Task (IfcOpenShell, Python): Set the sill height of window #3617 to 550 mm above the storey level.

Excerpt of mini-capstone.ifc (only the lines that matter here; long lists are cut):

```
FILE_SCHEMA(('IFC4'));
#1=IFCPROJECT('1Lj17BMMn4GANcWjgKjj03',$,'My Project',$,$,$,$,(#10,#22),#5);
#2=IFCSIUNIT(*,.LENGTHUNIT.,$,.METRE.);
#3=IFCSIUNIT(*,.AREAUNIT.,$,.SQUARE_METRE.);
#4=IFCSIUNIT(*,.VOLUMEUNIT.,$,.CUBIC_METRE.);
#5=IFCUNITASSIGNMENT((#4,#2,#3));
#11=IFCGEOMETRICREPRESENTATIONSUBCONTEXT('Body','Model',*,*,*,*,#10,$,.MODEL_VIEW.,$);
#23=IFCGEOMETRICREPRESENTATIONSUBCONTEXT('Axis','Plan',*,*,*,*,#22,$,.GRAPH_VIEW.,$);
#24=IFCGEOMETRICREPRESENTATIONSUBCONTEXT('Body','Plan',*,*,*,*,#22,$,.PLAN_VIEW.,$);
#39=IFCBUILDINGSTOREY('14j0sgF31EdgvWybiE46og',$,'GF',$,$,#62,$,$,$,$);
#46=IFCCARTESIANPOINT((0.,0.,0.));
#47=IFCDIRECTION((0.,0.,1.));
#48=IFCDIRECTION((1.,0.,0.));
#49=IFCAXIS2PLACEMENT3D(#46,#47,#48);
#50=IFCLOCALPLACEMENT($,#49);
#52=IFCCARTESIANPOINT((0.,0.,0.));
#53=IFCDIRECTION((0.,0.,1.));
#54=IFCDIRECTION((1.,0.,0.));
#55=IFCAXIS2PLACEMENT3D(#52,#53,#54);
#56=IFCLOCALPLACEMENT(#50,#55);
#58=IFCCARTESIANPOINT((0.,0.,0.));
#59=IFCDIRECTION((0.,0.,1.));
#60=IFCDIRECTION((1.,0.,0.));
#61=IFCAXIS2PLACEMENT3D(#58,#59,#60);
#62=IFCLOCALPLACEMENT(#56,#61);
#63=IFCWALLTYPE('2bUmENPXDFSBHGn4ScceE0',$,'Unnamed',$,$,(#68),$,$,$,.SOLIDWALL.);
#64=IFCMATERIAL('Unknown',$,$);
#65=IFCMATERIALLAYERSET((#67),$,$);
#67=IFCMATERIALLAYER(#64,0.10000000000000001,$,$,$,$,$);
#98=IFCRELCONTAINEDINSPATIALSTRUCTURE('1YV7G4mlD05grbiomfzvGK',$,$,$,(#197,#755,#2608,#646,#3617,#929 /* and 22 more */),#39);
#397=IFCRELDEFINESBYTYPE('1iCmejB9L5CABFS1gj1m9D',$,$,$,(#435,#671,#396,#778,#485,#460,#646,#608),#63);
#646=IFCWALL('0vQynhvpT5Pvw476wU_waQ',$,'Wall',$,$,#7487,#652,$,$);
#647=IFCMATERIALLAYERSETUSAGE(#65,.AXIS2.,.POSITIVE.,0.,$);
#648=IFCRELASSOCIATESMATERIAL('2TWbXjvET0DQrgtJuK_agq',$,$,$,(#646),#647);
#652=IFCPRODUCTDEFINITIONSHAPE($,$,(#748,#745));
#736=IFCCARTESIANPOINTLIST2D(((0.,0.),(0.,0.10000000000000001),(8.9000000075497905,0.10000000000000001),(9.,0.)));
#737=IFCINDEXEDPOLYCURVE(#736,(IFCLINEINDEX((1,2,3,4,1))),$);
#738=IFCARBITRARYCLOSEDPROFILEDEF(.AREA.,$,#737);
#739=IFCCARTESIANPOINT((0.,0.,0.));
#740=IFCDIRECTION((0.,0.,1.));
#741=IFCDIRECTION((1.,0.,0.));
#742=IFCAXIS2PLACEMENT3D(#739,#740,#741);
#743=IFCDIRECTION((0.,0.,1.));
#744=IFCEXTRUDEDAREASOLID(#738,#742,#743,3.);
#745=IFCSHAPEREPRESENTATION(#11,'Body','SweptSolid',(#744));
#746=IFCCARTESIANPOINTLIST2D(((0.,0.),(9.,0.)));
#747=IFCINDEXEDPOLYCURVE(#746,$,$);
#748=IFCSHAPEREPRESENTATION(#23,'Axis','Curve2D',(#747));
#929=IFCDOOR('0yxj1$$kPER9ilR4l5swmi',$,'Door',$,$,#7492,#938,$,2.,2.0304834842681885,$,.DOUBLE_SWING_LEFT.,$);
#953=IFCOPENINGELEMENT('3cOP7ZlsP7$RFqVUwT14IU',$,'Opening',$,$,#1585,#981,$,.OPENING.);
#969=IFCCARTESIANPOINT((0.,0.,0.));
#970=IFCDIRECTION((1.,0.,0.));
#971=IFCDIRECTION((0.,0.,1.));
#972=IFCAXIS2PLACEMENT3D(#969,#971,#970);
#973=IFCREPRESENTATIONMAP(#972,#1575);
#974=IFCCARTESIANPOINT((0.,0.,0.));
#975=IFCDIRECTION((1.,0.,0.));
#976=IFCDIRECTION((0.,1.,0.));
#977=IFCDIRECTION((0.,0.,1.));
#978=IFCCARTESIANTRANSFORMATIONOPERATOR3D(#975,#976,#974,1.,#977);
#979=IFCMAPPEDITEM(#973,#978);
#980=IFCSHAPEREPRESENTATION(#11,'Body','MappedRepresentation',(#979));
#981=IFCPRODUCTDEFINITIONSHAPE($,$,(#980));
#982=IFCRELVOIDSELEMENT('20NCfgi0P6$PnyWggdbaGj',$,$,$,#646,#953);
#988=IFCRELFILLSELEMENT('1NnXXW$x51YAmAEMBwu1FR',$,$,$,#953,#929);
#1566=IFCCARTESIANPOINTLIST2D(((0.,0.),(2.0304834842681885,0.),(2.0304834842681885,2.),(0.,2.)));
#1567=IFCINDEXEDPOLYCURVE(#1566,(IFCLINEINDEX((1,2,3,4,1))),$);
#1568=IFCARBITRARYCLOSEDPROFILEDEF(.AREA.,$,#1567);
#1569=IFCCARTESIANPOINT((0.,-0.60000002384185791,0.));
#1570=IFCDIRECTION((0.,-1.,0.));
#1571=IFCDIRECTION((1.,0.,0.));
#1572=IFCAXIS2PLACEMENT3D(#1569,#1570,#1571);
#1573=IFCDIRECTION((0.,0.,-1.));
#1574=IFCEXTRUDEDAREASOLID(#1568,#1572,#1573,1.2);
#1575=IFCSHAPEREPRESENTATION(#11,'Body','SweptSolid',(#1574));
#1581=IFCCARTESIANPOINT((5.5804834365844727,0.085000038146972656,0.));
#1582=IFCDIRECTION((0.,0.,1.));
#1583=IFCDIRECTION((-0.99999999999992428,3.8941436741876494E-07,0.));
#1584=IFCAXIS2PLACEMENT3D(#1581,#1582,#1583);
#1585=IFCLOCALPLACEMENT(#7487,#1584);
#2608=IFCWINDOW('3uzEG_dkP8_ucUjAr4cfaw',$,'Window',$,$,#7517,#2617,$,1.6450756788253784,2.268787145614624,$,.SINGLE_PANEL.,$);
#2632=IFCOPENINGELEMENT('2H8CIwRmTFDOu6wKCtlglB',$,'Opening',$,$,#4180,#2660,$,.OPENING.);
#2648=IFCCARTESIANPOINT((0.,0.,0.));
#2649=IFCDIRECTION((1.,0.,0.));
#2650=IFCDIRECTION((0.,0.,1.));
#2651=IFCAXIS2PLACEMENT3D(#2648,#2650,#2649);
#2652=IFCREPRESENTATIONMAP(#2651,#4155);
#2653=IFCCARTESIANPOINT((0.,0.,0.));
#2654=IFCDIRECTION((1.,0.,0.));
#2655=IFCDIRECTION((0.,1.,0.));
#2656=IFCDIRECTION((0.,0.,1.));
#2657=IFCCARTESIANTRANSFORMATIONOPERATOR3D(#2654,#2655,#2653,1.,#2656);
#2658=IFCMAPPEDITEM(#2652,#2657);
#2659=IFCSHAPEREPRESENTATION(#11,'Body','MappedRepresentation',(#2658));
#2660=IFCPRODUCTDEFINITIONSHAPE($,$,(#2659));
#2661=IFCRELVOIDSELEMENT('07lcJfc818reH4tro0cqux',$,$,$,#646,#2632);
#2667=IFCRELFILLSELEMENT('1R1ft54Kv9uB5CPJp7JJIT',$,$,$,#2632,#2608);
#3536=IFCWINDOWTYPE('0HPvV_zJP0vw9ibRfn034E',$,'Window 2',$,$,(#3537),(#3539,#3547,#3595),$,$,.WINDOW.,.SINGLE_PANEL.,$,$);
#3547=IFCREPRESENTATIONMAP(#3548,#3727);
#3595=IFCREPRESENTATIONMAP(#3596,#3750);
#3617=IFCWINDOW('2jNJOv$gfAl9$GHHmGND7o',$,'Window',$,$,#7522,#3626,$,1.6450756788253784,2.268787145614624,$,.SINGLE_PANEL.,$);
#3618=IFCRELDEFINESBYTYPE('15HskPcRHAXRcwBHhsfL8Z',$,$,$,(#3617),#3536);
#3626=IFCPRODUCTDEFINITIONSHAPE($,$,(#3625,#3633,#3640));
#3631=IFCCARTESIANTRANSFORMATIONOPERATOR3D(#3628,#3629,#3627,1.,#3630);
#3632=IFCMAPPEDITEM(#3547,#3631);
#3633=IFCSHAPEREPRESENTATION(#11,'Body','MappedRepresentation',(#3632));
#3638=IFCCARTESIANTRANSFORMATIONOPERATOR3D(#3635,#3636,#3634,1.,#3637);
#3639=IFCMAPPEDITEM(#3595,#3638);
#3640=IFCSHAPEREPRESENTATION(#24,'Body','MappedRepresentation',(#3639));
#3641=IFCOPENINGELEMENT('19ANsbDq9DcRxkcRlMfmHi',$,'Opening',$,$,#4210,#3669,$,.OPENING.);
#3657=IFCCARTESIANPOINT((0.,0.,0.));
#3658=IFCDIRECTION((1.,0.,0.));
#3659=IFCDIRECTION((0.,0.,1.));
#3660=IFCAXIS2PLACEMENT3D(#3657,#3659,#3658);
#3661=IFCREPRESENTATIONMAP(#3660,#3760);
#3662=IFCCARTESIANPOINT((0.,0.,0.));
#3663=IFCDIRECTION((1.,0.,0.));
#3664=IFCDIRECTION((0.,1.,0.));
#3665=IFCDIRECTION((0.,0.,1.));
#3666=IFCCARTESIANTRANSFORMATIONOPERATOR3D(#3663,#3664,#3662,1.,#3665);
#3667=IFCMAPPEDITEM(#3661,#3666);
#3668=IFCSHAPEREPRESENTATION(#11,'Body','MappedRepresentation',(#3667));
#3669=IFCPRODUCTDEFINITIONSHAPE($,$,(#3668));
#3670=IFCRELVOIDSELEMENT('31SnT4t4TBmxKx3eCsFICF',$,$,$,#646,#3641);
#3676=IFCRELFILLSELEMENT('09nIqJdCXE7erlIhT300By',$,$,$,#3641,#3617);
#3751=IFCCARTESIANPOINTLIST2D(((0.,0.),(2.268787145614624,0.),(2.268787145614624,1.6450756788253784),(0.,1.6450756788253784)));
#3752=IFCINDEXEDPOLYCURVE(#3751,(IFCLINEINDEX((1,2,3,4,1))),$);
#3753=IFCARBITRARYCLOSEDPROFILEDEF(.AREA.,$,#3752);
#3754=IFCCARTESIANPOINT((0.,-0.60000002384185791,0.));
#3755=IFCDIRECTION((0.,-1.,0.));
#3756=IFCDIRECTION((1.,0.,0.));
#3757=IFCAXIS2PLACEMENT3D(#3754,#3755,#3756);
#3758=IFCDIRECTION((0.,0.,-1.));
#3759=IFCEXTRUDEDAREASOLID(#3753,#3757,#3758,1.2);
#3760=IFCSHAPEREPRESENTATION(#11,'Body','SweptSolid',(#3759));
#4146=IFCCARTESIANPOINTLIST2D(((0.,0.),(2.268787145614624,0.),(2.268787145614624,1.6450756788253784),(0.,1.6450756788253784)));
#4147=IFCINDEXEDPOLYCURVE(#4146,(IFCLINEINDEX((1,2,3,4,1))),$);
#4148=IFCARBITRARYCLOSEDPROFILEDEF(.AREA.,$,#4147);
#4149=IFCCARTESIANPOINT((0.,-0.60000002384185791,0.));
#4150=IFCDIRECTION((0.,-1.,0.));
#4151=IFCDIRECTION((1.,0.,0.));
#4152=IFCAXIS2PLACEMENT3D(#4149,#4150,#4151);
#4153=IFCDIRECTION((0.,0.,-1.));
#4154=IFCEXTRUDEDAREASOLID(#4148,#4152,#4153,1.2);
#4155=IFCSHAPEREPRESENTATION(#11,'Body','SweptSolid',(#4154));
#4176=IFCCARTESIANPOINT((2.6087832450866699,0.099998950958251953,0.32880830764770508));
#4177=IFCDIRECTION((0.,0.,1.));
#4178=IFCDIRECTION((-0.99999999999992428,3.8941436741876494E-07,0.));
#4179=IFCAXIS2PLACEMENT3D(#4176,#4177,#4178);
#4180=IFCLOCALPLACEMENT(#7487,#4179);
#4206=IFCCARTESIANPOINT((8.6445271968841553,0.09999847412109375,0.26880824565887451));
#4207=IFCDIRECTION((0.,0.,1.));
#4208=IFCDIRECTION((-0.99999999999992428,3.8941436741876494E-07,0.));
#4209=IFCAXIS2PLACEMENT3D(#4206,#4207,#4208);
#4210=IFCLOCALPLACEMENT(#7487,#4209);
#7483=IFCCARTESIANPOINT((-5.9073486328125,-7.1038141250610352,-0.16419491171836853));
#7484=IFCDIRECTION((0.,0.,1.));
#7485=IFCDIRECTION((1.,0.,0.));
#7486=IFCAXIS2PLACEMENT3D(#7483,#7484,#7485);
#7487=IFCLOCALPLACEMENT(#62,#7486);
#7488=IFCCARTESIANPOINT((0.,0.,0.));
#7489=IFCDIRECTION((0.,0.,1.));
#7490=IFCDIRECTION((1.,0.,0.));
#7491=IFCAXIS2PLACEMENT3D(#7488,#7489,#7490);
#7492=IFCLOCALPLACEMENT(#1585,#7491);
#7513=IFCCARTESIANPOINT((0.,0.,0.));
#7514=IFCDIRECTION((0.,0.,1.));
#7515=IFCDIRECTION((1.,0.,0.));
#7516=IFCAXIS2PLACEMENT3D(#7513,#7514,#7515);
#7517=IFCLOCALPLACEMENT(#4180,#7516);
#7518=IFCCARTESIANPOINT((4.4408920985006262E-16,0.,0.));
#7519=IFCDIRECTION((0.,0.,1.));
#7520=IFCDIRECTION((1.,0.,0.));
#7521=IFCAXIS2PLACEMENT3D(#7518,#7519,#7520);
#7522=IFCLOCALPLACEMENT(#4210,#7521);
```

```python
import numpy as np
import ifcopenshell
import ifcopenshell.api.geometry
import ifcopenshell.geom
import ifcopenshell.util.element
import ifcopenshell.util.placement
import ifcopenshell.util.shape
import ifcopenshell.util.unit

model = ifcopenshell.open("mini-capstone.ifc")
unit_scale = ifcopenshell.util.unit.calculate_unit_scale(model)

window = model.by_id(3617)
opening = window.FillsVoids[0].RelatingOpeningElement
storey = ifcopenshell.util.element.get_container(window, ifc_class="IfcBuildingStorey")
level = ifcopenshell.util.placement.get_local_placement(storey.ObjectPlacement)[2, 3]

# The opening's origin need not be at the sill, so measure its lowest point.
shape = ifcopenshell.geom.create_shape(ifcopenshell.geom.settings(), opening)
bottom = ifcopenshell.util.shape.get_shape_bottom_elevation(shape, shape.geometry) / unit_scale
dz = level + 0.55 / unit_scale - bottom

shift = np.array([0.0, 0.0, dz])
# The window is placed relative to its opening, so it follows when the opening moves.
matrix = ifcopenshell.util.placement.get_local_placement(opening.ObjectPlacement)
matrix[:3, 3] += shift
ifcopenshell.api.geometry.edit_object_placement(
    model, product=opening, matrix=matrix, is_si=False, should_transform_children=True
)

print(f"moved by {dz * unit_scale:+.3f} m")

model.write("mini-capstone_edited.ifc")
```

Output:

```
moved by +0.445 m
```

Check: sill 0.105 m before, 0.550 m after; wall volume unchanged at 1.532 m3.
